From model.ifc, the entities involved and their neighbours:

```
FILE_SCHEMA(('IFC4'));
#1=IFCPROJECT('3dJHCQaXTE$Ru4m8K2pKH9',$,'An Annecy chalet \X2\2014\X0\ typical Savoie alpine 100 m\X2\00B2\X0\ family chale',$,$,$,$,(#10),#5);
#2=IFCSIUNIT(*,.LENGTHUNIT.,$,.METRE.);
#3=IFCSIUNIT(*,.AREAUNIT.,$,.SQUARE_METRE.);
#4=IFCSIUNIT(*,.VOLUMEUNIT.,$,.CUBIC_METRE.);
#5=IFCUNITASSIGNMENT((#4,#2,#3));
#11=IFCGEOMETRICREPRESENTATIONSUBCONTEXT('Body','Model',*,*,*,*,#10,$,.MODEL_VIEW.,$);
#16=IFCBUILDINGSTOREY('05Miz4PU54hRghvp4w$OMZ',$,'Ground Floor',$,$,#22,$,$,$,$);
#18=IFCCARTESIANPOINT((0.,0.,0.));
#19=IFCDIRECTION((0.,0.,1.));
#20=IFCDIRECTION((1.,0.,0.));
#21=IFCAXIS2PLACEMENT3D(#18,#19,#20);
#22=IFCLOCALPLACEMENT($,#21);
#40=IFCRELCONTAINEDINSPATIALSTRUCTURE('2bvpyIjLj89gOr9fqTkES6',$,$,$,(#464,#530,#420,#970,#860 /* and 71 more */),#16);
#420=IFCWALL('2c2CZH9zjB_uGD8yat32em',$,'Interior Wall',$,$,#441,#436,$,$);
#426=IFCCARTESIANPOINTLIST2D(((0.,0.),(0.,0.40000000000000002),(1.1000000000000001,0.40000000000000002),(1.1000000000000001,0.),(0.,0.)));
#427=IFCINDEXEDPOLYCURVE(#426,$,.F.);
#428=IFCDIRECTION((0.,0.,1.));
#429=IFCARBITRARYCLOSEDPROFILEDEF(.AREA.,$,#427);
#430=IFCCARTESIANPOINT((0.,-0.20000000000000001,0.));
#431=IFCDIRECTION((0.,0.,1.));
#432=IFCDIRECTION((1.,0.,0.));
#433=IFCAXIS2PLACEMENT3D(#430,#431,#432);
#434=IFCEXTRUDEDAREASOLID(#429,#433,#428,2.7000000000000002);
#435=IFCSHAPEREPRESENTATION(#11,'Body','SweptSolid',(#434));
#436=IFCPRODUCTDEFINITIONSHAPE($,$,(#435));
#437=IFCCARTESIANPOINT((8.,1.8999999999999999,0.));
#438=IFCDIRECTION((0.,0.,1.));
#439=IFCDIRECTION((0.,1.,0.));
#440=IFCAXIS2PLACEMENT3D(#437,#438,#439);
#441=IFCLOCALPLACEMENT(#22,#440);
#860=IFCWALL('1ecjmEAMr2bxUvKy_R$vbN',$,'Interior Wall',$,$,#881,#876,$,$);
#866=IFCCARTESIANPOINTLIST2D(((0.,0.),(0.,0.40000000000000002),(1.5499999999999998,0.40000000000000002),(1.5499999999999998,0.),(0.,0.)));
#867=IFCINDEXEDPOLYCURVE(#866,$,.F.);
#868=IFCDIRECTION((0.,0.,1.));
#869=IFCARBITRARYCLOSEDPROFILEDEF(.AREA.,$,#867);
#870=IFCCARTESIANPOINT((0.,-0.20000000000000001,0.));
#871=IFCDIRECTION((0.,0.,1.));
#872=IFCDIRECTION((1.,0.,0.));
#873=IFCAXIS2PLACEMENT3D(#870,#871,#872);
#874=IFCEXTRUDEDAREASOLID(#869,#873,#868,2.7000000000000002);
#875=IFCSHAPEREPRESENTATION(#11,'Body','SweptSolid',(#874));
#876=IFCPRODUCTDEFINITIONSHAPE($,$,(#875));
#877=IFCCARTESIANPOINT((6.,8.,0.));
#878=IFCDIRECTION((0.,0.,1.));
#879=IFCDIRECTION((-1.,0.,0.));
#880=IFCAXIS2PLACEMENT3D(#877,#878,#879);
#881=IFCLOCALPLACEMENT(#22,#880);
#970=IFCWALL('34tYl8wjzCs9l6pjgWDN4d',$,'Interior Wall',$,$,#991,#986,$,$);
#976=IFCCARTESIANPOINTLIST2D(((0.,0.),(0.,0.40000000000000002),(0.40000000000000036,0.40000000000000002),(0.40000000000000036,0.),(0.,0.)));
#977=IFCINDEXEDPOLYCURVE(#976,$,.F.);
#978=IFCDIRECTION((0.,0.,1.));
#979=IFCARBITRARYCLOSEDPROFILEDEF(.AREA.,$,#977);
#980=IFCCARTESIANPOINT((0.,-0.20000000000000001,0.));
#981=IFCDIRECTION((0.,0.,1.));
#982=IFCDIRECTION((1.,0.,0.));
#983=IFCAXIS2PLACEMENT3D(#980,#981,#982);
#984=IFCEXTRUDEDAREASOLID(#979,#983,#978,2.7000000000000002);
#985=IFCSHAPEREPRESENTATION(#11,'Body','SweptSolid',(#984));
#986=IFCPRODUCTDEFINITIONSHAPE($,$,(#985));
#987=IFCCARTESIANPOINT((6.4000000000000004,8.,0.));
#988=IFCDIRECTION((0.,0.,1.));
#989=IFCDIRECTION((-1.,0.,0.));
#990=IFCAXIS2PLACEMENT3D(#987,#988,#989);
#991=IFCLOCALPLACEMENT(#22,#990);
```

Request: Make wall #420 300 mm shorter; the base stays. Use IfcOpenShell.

```python
import ifcopenshell
import ifcopenshell.geom
import ifcopenshell.util.representation
import ifcopenshell.util.shape
import ifcopenshell.util.unit

model = ifcopenshell.open("model.ifc")
unit_scale = ifcopenshell.util.unit.calculate_unit_scale(model)
settings = ifcopenshell.geom.settings()


def volume(element):
    """Net volume in cubic metres, openings subtracted."""
    shape = ifcopenshell.geom.create_shape(settings, element)
    return ifcopenshell.util.shape.get_volume(shape.geometry)


wall = model.by_guid("2c2CZH9zjB_uGD8yat32em")
before = volume(wall)

body = ifcopenshell.util.representation.get_representation(wall, "Model", "Body")
solid = body.Items[0]
old_height = solid.Depth
solid.Depth -= 0.3 / unit_scale
after = volume(wall)

print(f"height {old_height:g} -> {solid.Depth:g}, volume {before:.3f} -> {after:.3f} m3")

model.write("model_v2.ifc")
```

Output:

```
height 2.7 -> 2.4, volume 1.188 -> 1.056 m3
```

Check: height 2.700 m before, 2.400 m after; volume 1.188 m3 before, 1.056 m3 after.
